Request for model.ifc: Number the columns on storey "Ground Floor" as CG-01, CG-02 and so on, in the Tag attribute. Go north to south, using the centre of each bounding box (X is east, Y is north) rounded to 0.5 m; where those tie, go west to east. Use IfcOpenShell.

First a look at what the model holds.

```python
import ifcopenshell
import ifcopenshell.util.element
import ifcopenshell.util.placement

model = ifcopenshell.open("model.ifc")
print(model.schema)
storey = next(s for s in model.by_type("IfcBuildingStorey") if s.Name == "Ground Floor")
columns = [e for e in ifcopenshell.util.element.get_decomposition(storey) if e.is_a("IfcColumn")]
for e in sorted(columns, key=lambda e: e.id()):
    origin = ifcopenshell.util.placement.get_local_placement(e.ObjectPlacement)[:3, 3]
    print(e.id(), e.Tag, e.Name, origin.round(2) + 0.0, sep=" | ")
```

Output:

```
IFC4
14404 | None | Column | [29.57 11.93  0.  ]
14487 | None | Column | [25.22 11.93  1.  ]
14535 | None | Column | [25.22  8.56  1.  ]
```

```python
import ifcopenshell
import ifcopenshell.geom
import ifcopenshell.util.element
import ifcopenshell.util.shape

model = ifcopenshell.open("model.ifc")
settings = ifcopenshell.geom.settings()
settings.set("use-world-coords", True)


def centre(element):
    shape = ifcopenshell.geom.create_shape(settings, element)
    return ifcopenshell.util.shape.get_bbox_centroid(shape.geometry)


storey = next(s for s in model.by_type("IfcBuildingStorey") if s.Name == "Ground Floor")
columns = [e for e in ifcopenshell.util.element.get_decomposition(storey) if e.is_a("IfcColumn")]

# Insertion points can sit at a corner or the storey origin, so sort by the geometry (in metres).
centres = {e: centre(e) for e in columns}
columns.sort(key=lambda e: (-round(centres[e][1] / 0.5), centres[e][0]))

for i, e in enumerate(columns, start=1):
    number = f"CG-{i:02d}"
    e.Tag = number
    print(e.id(), number)

model.write("model_edited.ifc")
```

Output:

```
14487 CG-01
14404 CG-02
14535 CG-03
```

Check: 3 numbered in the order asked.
